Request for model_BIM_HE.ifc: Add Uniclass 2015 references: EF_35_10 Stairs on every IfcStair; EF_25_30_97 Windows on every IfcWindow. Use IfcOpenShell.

First a look at what the model holds.

```python
import ifcopenshell

model = ifcopenshell.open("model_BIM_HE.ifc")
print(model.schema)
print("classifications:", [c.Name for c in model.by_type("IfcClassification")])
for ifc_class in ("IfcDoor", "IfcRoof", "IfcStair", "IfcWall", "IfcWindow"):
    print(ifc_class, len(model.by_type(ifc_class)))
```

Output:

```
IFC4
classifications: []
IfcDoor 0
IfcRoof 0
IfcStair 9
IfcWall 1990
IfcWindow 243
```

```python
import ifcopenshell
import ifcopenshell.api.classification

model = ifcopenshell.open("model_BIM_HE.ifc")

system = ifcopenshell.api.classification.add_classification(model, classification="Uniclass 2015")

codes = {
    "IfcStair": ("EF_35_10", "Stairs"),
    "IfcWindow": ("EF_25_30_97", "Windows"),
}
for ifc_class, (code, name) in codes.items():
    products = model.by_type(ifc_class)
    ifcopenshell.api.classification.add_reference(
        model, products=products, classification=system, identification=code, name=name
    )
    print(code, len(products))

model.write("model_BIM_HE_updated.ifc")
```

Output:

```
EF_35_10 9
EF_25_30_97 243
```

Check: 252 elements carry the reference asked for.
